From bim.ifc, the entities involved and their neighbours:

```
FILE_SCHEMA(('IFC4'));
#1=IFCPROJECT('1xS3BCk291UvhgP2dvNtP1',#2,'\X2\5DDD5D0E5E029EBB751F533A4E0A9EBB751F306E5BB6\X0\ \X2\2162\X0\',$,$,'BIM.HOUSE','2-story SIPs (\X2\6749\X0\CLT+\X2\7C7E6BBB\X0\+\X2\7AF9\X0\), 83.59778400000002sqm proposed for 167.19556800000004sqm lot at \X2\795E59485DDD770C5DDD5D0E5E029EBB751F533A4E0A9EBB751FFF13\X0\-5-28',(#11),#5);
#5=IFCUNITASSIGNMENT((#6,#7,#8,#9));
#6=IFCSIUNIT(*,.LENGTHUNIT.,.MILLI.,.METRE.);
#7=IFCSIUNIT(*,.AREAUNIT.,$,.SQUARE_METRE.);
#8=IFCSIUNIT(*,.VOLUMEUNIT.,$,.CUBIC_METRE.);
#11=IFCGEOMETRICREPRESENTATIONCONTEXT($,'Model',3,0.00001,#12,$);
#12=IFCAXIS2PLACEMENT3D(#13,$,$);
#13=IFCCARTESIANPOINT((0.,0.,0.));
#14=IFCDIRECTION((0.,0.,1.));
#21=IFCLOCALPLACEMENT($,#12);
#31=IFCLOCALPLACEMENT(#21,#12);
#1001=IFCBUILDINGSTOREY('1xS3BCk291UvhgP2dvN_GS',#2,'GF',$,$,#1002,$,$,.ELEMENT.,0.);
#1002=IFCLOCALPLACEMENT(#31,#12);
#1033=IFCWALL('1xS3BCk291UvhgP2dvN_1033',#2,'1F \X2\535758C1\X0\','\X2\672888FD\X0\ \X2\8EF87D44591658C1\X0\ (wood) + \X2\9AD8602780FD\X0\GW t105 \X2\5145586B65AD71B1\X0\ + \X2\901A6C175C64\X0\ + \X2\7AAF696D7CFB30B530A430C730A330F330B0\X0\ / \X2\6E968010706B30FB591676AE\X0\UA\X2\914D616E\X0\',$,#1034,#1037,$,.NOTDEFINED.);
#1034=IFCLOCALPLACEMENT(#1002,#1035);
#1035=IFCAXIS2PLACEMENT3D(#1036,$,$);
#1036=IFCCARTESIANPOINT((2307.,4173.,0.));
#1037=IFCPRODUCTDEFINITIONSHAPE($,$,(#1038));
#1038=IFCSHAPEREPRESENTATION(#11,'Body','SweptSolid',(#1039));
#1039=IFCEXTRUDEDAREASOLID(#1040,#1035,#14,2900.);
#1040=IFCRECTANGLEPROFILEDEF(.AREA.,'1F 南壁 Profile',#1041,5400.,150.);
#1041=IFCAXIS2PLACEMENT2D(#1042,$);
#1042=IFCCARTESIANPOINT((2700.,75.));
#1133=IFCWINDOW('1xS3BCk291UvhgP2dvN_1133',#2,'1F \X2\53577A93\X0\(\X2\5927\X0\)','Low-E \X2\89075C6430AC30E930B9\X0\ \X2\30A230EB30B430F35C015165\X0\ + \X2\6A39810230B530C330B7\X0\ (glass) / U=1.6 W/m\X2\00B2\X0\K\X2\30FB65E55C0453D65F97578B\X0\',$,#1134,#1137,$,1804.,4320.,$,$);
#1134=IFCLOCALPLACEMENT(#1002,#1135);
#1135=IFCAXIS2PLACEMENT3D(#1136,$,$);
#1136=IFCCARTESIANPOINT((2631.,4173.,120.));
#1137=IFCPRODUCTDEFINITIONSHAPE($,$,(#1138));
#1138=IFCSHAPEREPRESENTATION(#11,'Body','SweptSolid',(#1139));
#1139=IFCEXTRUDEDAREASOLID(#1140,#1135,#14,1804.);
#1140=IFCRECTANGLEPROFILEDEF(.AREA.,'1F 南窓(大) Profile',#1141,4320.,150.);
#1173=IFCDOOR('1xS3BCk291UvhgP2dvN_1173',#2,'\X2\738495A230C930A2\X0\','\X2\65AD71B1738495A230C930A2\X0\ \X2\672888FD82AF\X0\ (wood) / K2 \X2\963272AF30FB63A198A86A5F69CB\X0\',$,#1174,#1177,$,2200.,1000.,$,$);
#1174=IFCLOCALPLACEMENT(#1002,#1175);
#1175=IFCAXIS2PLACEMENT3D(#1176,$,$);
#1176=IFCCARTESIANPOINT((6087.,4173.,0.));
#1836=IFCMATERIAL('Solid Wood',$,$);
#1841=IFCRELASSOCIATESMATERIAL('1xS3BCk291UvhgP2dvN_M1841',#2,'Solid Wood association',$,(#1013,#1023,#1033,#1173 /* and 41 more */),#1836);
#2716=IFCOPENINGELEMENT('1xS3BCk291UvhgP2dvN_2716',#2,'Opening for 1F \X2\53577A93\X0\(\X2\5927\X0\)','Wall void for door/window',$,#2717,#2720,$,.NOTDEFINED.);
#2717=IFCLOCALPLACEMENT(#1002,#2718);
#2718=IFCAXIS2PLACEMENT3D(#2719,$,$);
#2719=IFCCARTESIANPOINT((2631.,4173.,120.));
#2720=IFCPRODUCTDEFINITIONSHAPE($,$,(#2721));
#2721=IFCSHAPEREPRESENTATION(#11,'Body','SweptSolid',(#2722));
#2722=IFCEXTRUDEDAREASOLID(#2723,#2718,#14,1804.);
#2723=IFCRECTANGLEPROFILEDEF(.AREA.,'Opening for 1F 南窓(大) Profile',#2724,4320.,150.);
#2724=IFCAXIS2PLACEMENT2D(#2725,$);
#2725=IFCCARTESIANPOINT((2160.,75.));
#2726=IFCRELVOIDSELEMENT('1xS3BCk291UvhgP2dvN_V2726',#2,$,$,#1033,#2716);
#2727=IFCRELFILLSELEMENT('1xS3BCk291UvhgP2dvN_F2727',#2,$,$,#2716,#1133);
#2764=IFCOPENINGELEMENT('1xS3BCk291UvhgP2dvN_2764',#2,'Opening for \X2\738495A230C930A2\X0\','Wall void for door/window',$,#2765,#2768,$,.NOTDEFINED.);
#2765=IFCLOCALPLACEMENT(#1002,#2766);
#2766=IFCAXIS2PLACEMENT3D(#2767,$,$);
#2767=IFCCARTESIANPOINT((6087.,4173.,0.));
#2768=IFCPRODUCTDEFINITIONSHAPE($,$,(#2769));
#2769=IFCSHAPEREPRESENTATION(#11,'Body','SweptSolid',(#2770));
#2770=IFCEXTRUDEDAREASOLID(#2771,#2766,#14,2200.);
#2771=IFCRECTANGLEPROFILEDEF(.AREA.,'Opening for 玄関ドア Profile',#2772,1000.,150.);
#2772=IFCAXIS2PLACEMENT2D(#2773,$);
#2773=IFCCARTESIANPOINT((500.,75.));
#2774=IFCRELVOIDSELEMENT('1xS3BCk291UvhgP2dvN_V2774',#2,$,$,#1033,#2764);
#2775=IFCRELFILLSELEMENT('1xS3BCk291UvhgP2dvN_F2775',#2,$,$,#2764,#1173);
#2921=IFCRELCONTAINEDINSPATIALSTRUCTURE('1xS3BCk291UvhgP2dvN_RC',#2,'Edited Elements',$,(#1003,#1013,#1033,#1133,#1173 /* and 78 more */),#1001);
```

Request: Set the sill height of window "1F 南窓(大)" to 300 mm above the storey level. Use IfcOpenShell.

```python
import numpy as np
import ifcopenshell
import ifcopenshell.api.geometry
import ifcopenshell.geom
import ifcopenshell.util.element
import ifcopenshell.util.placement
import ifcopenshell.util.shape
import ifcopenshell.util.unit

model = ifcopenshell.open("bim.ifc")
unit_scale = ifcopenshell.util.unit.calculate_unit_scale(model)

window = model.by_guid("1xS3BCk291UvhgP2dvN_1133")
opening = window.FillsVoids[0].RelatingOpeningElement
storey = ifcopenshell.util.element.get_container(window, ifc_class="IfcBuildingStorey")
level = ifcopenshell.util.placement.get_local_placement(storey.ObjectPlacement)[2, 3]

# The opening's origin need not be at the sill, so measure its lowest point.
shape = ifcopenshell.geom.create_shape(ifcopenshell.geom.settings(), opening)
bottom = ifcopenshell.util.shape.get_shape_bottom_elevation(shape, shape.geometry) / unit_scale
dz = level + 0.3 / unit_scale - bottom

shift = np.array([0.0, 0.0, dz])
# The window is not placed relative to its opening, so move both.
for product in (opening, window):
    matrix = ifcopenshell.util.placement.get_local_placement(product.ObjectPlacement)
    matrix[:3, 3] += shift
    ifcopenshell.api.geometry.edit_object_placement(model, product=product, matrix=matrix, is_si=False)

print(f"moved by {dz * unit_scale:+.3f} m")

model.write("bim_edited.ifc")
```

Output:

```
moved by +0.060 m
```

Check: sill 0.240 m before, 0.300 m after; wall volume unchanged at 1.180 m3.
